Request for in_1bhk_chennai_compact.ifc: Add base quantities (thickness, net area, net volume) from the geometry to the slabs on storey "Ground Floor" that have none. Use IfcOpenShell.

First a look at what the model holds.

```python
import ifcopenshell
import ifcopenshell.util.element
import ifcopenshell.util.unit

model = ifcopenshell.open("in_1bhk_chennai_compact.ifc")
print(model.schema)
for unit_type in ("LENGTHUNIT", "AREAUNIT", "VOLUMEUNIT"):
    print(unit_type, ifcopenshell.util.unit.calculate_unit_scale(model, unit_type))
storey = next(s for s in model.by_type("IfcBuildingStorey") if s.Name == "Ground Floor")
slabs = [e for e in ifcopenshell.util.element.get_decomposition(storey) if e.is_a("IfcSlab")]
for e in sorted(slabs, key=lambda e: e.id()):
    print(e.id(), e.is_a(), e.Name, list(ifcopenshell.util.element.get_psets(e, qtos_only=True)), sep=" | ")
```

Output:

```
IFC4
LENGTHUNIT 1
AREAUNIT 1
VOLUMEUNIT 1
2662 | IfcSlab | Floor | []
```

```python
import ifcopenshell
import ifcopenshell.api.pset
import ifcopenshell.geom
import ifcopenshell.util.element
import ifcopenshell.util.shape
import ifcopenshell.util.unit

model = ifcopenshell.open("in_1bhk_chennai_compact.ifc")
unit_scale = ifcopenshell.util.unit.calculate_unit_scale(model)
area_scale = ifcopenshell.util.unit.calculate_unit_scale(model, "AREAUNIT")
volume_scale = ifcopenshell.util.unit.calculate_unit_scale(model, "VOLUMEUNIT")
settings = ifcopenshell.geom.settings()

storey = next(s for s in model.by_type("IfcBuildingStorey") if s.Name == "Ground Floor")
slabs = [e for e in ifcopenshell.util.element.get_decomposition(storey) if e.is_a("IfcSlab")]

for e in sorted(slabs, key=lambda e: e.id()):
    if ifcopenshell.util.element.get_psets(e, qtos_only=True, should_inherit=False):
        continue
    # Geometry comes back in metres, in the element's own axes.
    shape = ifcopenshell.geom.create_shape(settings, e)
    values = {
        "Width": ifcopenshell.util.shape.get_z(shape.geometry) / unit_scale,
        "NetArea": ifcopenshell.util.shape.get_footprint_area(shape.geometry) / area_scale,
        "NetVolume": ifcopenshell.util.shape.get_volume(shape.geometry) / volume_scale,
    }
    qto = ifcopenshell.api.pset.add_qto(model, product=e, name="Qto_SlabBaseQuantities")
    ifcopenshell.api.pset.edit_qto(model, qto=qto, properties=values)
    print(e.id(), {k: round(v, 3) for k, v in values.items()})

model.write("in_1bhk_chennai_compact_edited.ifc")
```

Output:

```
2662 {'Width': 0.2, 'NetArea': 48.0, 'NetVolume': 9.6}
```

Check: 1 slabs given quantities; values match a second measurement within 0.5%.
